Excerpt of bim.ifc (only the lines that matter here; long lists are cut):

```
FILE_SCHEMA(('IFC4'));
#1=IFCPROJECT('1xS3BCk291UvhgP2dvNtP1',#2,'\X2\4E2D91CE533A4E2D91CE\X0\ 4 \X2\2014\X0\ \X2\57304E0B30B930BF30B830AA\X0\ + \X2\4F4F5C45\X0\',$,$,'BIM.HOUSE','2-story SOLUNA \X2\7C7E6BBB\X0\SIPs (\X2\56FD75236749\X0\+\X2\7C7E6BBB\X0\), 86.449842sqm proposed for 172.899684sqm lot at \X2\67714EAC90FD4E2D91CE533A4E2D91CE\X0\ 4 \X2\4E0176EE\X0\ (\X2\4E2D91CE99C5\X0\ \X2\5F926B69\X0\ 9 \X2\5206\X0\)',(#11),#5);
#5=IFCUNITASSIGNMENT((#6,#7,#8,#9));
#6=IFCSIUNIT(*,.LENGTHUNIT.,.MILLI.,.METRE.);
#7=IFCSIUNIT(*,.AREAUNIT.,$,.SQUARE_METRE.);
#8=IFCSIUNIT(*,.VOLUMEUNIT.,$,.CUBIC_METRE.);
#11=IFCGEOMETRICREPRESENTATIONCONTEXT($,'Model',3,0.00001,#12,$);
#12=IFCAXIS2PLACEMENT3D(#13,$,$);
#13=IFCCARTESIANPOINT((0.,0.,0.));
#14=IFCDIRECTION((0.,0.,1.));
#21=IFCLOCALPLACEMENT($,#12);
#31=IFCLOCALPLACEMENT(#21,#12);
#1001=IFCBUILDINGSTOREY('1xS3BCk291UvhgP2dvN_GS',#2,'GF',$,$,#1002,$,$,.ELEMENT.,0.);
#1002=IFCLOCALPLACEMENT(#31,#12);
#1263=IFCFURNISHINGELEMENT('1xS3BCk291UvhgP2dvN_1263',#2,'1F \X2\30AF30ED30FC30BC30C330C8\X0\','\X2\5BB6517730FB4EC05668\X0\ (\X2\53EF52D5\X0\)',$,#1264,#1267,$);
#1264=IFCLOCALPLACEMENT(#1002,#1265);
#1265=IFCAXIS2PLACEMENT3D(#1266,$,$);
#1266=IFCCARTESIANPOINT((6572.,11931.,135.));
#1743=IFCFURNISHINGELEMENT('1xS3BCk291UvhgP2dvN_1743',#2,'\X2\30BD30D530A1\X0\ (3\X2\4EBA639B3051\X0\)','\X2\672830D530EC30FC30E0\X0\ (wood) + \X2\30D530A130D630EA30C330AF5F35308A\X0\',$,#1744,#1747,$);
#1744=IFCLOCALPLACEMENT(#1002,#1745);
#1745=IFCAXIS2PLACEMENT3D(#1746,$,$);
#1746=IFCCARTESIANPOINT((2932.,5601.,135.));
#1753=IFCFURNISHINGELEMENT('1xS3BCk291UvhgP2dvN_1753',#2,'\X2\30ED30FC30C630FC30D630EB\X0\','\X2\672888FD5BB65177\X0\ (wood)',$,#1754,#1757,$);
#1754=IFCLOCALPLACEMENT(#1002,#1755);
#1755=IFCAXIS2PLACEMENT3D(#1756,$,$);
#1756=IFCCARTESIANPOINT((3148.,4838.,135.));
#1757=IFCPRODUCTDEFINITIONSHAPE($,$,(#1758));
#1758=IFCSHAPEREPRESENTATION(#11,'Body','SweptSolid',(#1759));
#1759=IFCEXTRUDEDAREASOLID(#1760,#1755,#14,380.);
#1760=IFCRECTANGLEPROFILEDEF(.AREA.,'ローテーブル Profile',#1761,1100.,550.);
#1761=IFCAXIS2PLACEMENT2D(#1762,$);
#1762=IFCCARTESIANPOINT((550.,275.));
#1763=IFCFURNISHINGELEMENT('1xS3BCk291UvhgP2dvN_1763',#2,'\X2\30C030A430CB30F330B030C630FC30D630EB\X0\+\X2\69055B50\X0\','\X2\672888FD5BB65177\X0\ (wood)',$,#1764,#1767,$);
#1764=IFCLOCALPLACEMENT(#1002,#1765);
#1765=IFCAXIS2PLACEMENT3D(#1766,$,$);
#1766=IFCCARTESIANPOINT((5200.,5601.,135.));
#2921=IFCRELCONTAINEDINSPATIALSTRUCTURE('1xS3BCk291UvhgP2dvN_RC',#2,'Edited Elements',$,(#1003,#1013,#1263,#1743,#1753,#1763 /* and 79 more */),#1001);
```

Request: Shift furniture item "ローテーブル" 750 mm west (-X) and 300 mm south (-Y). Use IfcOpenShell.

```python
import ifcopenshell
import ifcopenshell.api.geometry
import ifcopenshell.util.placement
import ifcopenshell.util.unit

model = ifcopenshell.open("bim.ifc")
unit_scale = ifcopenshell.util.unit.calculate_unit_scale(model)

item = model.by_guid("1xS3BCk291UvhgP2dvN_1753")
matrix = ifcopenshell.util.placement.get_local_placement(item.ObjectPlacement)
matrix[0, 3] -= 0.75 / unit_scale
matrix[1, 3] -= 0.3 / unit_scale
ifcopenshell.api.geometry.edit_object_placement(model, product=item, matrix=matrix, is_si=False)

print(ifcopenshell.util.placement.get_local_placement(item.ObjectPlacement).round(3) + 0.0)

model.write("bim_updated.ifc")
```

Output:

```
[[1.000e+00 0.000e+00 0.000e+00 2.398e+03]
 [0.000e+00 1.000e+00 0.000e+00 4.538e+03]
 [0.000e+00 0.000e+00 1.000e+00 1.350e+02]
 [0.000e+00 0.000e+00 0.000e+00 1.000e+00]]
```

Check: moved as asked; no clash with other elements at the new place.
